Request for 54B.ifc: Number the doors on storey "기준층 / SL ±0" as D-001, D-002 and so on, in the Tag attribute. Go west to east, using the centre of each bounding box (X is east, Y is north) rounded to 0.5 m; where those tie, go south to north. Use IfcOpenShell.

First a look at what the model holds.

```python
import ifcopenshell
import ifcopenshell.util.element
import ifcopenshell.util.placement

model = ifcopenshell.open("54B.ifc")
print(model.schema)
storey = next(s for s in model.by_type("IfcBuildingStorey") if s.Name == "기준층 / SL ±0")
doors = [e for e in ifcopenshell.util.element.get_decomposition(storey) if e.is_a("IfcDoor")]
for e in sorted(doors, key=lambda e: e.id()):
    origin = ifcopenshell.util.placement.get_local_placement(e.ObjectPlacement)[:3, 3]
    print(e.id(), e.Tag, e.Name, origin.round(2) + 0.0, sep=" | ")
```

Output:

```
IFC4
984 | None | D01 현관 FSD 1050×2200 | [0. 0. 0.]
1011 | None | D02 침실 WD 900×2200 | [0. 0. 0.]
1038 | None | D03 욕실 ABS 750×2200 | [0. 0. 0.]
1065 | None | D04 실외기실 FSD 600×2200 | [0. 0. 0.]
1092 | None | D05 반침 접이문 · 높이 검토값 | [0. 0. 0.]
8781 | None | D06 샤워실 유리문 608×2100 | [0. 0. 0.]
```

```python
import ifcopenshell
import ifcopenshell.geom
import ifcopenshell.util.element
import ifcopenshell.util.shape

model = ifcopenshell.open("54B.ifc")
settings = ifcopenshell.geom.settings()
settings.set("use-world-coords", True)


def centre(element):
    shape = ifcopenshell.geom.create_shape(settings, element)
    return ifcopenshell.util.shape.get_bbox_centroid(shape.geometry)


storey = next(s for s in model.by_type("IfcBuildingStorey") if s.Name == "기준층 / SL ±0")
doors = [e for e in ifcopenshell.util.element.get_decomposition(storey) if e.is_a("IfcDoor")]

# Insertion points can sit at a corner or the storey origin, so sort by the geometry (in metres).
centres = {e: centre(e) for e in doors}
doors.sort(key=lambda e: (round(centres[e][0] / 0.5), centres[e][1]))

for i, e in enumerate(doors, start=1):
    number = f"D-0{i:02d}"
    e.Tag = number
    print(e.id(), number)

model.write("54B_rev.ifc")
```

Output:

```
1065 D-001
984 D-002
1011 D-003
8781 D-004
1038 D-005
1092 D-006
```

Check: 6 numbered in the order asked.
